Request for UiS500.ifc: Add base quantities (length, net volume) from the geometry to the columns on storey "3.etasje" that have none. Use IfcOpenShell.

First a look at what the model holds.

```python
import ifcopenshell
import ifcopenshell.util.element
import ifcopenshell.util.unit

model = ifcopenshell.open("UiS500.ifc")
print(model.schema)
for unit_type in ("LENGTHUNIT", "AREAUNIT", "VOLUMEUNIT"):
    print(unit_type, ifcopenshell.util.unit.calculate_unit_scale(model, unit_type))
storey = next(s for s in model.by_type("IfcBuildingStorey") if s.Name == "3.etasje")
columns = [e for e in ifcopenshell.util.element.get_decomposition(storey) if e.is_a("IfcColumn")]
for e in sorted(columns, key=lambda e: e.id()):
    print(e.id(), e.is_a(), e.Name, list(ifcopenshell.util.element.get_psets(e, qtos_only=True)), sep=" | ")
```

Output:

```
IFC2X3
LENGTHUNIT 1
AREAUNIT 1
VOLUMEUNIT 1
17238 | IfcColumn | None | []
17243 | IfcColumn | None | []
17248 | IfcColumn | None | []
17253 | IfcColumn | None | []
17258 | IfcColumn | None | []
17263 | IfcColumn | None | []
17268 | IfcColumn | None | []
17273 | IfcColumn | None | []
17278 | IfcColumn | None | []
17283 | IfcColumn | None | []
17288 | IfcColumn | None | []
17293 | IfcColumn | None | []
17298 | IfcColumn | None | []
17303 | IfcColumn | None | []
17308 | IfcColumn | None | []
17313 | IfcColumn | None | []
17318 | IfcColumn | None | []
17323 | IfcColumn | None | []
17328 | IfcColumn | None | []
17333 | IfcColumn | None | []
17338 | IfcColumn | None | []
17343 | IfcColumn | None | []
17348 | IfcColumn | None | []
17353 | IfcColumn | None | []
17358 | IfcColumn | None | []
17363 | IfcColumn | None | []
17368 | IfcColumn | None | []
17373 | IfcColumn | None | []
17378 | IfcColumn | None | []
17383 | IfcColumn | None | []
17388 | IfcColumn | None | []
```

```python
import ifcopenshell
import ifcopenshell.api.pset
import ifcopenshell.geom
import ifcopenshell.util.element
import ifcopenshell.util.shape
import ifcopenshell.util.unit

model = ifcopenshell.open("UiS500.ifc")
unit_scale = ifcopenshell.util.unit.calculate_unit_scale(model)
volume_scale = ifcopenshell.util.unit.calculate_unit_scale(model, "VOLUMEUNIT")
settings = ifcopenshell.geom.settings()

storey = next(s for s in model.by_type("IfcBuildingStorey") if s.Name == "3.etasje")
columns = [e for e in ifcopenshell.util.element.get_decomposition(storey) if e.is_a("IfcColumn")]

for e in sorted(columns, key=lambda e: e.id()):
    if ifcopenshell.util.element.get_psets(e, qtos_only=True, should_inherit=False):
        continue
    # Geometry comes back in metres, in the element's own axes.
    shape = ifcopenshell.geom.create_shape(settings, e)
    values = {
        "Length": ifcopenshell.util.shape.get_z(shape.geometry) / unit_scale,
        "NetVolume": ifcopenshell.util.shape.get_volume(shape.geometry) / volume_scale,
    }
    qto = ifcopenshell.api.pset.add_qto(model, product=e, name="BaseQuantities")
    ifcopenshell.api.pset.edit_qto(model, qto=qto, properties=values)
    print(e.id(), {k: round(v, 3) for k, v in values.items()})

model.write("UiS500_v2.ifc")
```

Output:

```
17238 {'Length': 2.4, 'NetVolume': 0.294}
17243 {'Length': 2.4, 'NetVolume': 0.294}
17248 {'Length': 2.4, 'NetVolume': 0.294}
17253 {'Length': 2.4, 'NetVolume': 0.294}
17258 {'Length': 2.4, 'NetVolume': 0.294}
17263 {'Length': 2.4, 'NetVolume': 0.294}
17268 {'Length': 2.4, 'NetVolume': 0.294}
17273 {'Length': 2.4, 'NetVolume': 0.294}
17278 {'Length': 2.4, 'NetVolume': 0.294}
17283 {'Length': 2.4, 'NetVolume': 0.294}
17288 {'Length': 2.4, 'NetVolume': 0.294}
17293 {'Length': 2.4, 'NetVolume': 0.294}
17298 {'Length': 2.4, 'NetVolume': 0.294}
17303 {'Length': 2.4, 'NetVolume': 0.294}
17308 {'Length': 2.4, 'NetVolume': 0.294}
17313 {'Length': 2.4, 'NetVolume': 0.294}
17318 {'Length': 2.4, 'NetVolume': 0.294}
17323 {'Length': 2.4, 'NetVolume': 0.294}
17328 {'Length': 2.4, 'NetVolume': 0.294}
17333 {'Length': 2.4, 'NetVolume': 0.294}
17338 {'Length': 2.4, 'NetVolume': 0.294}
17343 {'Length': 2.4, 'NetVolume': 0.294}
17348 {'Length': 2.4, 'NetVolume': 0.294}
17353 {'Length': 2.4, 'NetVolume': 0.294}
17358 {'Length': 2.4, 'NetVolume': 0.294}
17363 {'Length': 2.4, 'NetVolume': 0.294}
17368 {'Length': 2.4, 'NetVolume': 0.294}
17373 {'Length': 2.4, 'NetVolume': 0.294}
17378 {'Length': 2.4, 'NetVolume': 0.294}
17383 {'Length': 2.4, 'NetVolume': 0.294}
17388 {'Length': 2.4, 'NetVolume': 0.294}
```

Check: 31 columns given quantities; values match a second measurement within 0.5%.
